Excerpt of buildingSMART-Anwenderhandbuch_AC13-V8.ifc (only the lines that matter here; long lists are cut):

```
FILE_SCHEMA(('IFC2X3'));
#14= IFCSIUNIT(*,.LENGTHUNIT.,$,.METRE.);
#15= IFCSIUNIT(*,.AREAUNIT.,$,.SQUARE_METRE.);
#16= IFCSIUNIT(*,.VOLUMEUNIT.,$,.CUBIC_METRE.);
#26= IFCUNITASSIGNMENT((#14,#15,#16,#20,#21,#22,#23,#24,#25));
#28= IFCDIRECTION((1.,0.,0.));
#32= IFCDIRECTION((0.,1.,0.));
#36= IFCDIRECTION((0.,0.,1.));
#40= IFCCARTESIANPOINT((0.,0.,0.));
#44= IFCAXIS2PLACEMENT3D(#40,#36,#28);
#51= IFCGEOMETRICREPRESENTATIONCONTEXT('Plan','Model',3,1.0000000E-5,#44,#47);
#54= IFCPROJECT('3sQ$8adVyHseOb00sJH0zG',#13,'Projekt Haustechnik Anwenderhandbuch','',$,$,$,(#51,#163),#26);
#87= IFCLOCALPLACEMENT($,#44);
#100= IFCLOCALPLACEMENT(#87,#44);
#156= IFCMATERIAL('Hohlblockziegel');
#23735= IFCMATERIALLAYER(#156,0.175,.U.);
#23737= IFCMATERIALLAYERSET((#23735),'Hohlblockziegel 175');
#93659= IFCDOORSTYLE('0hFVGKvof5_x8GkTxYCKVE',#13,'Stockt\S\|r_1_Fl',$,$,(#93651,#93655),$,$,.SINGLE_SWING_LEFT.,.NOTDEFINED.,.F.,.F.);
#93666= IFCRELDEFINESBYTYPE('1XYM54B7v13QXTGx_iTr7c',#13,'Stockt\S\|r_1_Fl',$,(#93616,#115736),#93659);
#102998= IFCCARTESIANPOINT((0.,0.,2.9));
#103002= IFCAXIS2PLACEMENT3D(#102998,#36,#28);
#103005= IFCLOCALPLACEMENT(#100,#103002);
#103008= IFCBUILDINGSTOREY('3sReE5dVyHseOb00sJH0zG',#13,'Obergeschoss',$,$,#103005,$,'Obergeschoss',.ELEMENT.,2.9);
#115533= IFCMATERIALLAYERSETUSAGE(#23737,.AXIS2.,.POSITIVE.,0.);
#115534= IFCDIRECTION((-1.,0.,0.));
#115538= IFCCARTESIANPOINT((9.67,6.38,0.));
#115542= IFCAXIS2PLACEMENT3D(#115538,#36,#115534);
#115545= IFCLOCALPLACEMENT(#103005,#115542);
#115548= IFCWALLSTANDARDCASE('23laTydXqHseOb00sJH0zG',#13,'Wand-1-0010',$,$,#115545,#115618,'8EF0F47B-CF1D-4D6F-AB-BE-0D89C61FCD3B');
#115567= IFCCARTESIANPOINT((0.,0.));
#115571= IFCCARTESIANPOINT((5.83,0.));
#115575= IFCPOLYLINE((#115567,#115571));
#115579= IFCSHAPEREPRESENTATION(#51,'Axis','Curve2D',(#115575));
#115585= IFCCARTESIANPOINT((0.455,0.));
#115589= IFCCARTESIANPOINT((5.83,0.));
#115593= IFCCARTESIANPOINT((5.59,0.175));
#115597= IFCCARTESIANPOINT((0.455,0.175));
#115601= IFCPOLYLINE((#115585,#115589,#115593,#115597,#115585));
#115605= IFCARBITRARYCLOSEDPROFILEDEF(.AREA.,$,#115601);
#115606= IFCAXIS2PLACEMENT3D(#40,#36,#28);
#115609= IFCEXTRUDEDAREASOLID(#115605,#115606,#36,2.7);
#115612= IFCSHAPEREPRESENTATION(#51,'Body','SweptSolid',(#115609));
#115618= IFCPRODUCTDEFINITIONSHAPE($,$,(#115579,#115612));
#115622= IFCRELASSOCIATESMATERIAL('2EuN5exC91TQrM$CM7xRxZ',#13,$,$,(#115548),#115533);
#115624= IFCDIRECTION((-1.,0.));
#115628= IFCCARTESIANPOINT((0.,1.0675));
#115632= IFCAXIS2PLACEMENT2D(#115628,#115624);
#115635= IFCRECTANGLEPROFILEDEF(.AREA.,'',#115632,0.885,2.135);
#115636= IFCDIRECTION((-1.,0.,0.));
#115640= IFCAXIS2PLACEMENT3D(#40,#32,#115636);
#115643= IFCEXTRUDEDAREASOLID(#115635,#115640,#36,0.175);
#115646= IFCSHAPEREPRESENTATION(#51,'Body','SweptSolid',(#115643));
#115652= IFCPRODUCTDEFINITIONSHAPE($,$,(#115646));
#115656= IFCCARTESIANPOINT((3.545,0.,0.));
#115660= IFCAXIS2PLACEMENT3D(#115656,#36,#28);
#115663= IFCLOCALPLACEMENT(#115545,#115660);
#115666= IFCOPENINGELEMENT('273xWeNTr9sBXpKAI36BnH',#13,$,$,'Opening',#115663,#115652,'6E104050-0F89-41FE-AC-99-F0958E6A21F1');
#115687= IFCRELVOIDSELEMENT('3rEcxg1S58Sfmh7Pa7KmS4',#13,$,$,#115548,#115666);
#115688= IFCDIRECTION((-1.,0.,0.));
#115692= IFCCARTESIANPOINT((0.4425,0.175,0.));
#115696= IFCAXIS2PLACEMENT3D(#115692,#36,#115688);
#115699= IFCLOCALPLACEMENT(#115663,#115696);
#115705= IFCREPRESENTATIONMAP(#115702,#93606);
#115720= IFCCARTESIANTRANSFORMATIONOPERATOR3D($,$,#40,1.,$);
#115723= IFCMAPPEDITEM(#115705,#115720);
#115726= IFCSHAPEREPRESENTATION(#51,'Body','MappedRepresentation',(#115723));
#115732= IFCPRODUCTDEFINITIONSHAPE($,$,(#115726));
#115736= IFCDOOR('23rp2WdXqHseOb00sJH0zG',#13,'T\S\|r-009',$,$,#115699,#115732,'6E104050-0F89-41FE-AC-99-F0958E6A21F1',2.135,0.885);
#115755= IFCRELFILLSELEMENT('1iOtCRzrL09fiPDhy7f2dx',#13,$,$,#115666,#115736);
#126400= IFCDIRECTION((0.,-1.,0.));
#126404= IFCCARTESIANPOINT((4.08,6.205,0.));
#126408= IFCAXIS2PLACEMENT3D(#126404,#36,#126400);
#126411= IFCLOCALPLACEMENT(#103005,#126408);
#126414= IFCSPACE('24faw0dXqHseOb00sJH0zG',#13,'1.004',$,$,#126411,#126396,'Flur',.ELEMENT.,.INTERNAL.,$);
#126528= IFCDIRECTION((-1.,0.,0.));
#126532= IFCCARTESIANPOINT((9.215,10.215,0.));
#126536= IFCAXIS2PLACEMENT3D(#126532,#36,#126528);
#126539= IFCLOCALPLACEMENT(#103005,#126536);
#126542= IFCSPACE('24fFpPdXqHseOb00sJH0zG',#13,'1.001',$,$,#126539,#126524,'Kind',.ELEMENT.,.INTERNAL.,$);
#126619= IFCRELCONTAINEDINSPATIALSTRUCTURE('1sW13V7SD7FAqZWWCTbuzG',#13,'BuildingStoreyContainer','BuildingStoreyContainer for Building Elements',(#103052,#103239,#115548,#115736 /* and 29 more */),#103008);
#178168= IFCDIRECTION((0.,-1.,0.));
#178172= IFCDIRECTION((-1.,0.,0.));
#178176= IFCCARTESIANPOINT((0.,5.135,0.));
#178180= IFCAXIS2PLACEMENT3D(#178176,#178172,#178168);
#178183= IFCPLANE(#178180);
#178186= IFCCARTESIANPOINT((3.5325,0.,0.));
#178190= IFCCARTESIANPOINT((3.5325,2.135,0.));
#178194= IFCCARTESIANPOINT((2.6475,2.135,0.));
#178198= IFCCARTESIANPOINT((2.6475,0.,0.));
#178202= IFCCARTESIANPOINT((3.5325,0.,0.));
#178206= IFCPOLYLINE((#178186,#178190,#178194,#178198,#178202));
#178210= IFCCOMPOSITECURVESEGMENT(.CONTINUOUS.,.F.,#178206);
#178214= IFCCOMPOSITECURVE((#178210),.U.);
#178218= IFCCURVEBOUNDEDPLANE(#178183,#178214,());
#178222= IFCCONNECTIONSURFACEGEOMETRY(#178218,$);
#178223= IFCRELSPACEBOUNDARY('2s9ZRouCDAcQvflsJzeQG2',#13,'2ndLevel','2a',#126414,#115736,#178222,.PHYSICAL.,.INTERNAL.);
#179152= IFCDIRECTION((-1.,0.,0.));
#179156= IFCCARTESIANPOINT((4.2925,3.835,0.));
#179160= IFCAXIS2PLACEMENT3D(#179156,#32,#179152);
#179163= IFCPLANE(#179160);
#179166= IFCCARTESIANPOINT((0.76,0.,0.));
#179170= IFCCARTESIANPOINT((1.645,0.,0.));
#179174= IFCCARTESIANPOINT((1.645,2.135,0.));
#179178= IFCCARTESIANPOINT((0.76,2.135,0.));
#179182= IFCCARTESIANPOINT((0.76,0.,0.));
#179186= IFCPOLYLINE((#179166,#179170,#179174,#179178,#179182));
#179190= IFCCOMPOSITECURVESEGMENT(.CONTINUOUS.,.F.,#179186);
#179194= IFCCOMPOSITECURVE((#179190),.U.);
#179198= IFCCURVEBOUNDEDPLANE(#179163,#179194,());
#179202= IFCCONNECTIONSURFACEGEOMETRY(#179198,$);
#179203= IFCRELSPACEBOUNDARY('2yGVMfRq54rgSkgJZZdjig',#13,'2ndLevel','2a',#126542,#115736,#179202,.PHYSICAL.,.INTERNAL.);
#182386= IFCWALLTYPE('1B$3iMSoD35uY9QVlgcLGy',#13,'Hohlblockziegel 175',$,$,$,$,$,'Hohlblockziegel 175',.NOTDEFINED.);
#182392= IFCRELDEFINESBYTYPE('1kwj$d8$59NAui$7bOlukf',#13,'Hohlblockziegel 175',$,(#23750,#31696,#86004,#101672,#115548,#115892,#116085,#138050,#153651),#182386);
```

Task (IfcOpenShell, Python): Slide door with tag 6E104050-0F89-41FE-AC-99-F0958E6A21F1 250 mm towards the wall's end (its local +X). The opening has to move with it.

```python
import numpy as np
import ifcopenshell
import ifcopenshell.api.geometry
import ifcopenshell.util.placement
import ifcopenshell.util.unit

model = ifcopenshell.open("buildingSMART-Anwenderhandbuch_AC13-V8.ifc")
unit_scale = ifcopenshell.util.unit.calculate_unit_scale(model)

door = model.by_guid("23rp2WdXqHseOb00sJH0zG")
opening = door.FillsVoids[0].RelatingOpeningElement
wall = opening.VoidsElements[0].RelatingBuildingElement

wall_matrix = ifcopenshell.util.placement.get_local_placement(wall.ObjectPlacement)
shift = wall_matrix[:3, 0] * 0.25 / unit_scale
before = ifcopenshell.util.placement.get_local_placement(door.ObjectPlacement)[:3, 3].copy()

# The door is placed relative to its opening, so it follows when the opening moves.
matrix = ifcopenshell.util.placement.get_local_placement(opening.ObjectPlacement)
matrix[:3, 3] += shift
ifcopenshell.api.geometry.edit_object_placement(
    model, product=opening, matrix=matrix, is_si=False, should_transform_children=True
)

# Space boundary surfaces are stored in each space's coordinates; move them too.
for rel in door.ProvidesBoundaries:
    if not rel.ConnectionGeometry:
        continue
    surface = rel.ConnectionGeometry.SurfaceOnRelatingElement.BasisSurface
    space_matrix = ifcopenshell.util.placement.get_local_placement(rel.RelatingSpace.ObjectPlacement)
    point = np.array(surface.Position.Location.Coordinates) + space_matrix[:3, :3].T @ shift
    surface.Position = model.createIfcAxis2Placement3D(
        model.createIfcCartesianPoint(point.tolist()), surface.Position.Axis, surface.Position.RefDirection
    )

after = ifcopenshell.util.placement.get_local_placement(door.ObjectPlacement)[:3, 3]
print("door moved by", (after - before).round(3) + 0.0)

model.write("buildingSMART-Anwenderhandbuch_AC13-V8_v2.ifc")
```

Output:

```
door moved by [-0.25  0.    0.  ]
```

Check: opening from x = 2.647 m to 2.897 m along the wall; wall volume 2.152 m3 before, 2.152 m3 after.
